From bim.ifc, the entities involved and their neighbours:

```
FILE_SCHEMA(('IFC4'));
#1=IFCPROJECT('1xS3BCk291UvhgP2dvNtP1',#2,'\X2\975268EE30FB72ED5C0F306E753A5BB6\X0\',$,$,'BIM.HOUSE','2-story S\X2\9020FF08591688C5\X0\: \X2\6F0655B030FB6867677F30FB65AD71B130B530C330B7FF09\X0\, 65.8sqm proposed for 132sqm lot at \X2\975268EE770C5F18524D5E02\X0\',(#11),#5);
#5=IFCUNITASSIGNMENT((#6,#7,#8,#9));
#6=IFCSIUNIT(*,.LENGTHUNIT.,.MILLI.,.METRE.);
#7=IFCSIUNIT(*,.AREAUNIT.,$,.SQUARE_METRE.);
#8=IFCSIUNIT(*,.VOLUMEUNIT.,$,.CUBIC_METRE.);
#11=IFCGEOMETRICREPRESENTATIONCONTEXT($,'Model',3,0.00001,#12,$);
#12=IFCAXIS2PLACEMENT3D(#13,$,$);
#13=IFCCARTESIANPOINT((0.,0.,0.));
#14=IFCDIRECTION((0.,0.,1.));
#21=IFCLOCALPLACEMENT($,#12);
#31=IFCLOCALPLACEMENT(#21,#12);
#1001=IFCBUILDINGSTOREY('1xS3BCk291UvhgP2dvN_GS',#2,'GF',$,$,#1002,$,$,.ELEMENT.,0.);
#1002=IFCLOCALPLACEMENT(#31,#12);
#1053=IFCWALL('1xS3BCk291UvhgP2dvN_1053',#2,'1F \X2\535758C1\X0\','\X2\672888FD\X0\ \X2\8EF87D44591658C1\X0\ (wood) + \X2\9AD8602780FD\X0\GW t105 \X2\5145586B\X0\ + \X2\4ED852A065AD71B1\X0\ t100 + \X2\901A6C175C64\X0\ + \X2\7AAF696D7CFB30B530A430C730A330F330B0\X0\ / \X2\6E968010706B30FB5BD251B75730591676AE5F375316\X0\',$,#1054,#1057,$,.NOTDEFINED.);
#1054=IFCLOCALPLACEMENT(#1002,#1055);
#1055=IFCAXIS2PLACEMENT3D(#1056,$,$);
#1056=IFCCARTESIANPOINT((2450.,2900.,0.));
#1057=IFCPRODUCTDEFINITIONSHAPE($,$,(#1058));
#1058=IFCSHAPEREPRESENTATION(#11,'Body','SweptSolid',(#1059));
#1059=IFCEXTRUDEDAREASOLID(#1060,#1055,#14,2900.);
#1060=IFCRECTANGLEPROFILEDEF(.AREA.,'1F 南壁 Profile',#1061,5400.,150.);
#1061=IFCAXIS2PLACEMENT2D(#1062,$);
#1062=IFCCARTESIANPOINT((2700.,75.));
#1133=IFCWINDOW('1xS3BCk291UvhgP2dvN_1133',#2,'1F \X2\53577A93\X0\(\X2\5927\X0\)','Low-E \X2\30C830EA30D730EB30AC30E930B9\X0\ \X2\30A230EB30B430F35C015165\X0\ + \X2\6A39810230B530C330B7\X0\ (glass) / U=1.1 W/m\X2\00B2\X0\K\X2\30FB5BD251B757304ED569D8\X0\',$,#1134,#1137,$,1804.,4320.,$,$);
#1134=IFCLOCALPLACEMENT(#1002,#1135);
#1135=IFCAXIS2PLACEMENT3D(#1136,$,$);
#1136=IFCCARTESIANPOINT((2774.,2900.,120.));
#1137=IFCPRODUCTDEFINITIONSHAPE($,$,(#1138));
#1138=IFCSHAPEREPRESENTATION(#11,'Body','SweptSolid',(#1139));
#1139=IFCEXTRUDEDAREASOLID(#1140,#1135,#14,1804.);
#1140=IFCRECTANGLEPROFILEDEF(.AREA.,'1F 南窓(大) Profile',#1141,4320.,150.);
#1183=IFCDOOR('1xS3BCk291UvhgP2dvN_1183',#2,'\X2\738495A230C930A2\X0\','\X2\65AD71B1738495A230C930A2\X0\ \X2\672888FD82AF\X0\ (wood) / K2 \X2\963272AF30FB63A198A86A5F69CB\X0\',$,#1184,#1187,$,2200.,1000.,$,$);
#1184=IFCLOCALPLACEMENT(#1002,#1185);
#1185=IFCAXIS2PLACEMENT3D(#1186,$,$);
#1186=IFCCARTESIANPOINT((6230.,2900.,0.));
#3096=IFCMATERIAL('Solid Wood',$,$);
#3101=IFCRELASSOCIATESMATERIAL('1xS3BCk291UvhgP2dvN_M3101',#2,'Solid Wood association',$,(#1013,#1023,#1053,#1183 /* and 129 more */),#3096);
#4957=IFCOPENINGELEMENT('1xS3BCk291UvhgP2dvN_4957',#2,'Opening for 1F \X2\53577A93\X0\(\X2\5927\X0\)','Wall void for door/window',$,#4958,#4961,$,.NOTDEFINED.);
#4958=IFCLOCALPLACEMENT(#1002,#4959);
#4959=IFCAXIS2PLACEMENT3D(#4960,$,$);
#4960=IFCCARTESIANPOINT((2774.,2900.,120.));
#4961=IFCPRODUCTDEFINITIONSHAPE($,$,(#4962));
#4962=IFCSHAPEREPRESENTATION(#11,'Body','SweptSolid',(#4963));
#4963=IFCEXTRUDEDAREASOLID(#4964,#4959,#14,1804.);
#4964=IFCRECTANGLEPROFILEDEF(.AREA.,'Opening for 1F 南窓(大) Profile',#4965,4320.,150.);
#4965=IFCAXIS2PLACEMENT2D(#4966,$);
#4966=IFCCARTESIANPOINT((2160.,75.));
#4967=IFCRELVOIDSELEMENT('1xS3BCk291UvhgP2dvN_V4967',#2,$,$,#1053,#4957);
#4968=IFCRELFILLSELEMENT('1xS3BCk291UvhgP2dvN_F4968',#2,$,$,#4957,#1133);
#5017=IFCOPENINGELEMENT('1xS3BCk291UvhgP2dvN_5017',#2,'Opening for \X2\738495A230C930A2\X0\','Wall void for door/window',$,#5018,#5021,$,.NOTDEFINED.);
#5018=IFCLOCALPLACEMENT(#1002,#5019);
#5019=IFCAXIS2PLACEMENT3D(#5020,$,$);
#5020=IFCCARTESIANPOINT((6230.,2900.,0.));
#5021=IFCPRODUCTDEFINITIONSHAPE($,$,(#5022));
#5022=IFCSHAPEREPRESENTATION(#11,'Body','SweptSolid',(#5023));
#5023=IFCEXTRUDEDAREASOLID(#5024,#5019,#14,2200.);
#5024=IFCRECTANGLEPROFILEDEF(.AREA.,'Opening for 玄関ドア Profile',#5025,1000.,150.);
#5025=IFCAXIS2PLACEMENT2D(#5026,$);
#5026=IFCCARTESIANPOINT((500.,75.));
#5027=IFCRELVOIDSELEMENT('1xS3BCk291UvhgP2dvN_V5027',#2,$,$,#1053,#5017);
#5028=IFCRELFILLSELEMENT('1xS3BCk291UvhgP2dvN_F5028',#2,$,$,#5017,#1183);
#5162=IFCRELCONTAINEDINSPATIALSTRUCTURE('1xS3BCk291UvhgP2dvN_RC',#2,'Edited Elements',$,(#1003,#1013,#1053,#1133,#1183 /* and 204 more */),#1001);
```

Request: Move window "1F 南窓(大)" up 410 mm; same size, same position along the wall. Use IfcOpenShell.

```python
import numpy as np
import ifcopenshell
import ifcopenshell.api.geometry
import ifcopenshell.util.placement
import ifcopenshell.util.unit

model = ifcopenshell.open("bim.ifc")
unit_scale = ifcopenshell.util.unit.calculate_unit_scale(model)

window = model.by_guid("1xS3BCk291UvhgP2dvN_1133")
opening = window.FillsVoids[0].RelatingOpeningElement
dz = 0.41 / unit_scale

shift = np.array([0.0, 0.0, dz])
# The window is not placed relative to its opening, so move both.
for product in (opening, window):
    matrix = ifcopenshell.util.placement.get_local_placement(product.ObjectPlacement)
    matrix[:3, 3] += shift
    ifcopenshell.api.geometry.edit_object_placement(model, product=product, matrix=matrix, is_si=False)

print(f"moved by {dz * unit_scale:+.3f} m")

model.write("bim_edited.ifc")
```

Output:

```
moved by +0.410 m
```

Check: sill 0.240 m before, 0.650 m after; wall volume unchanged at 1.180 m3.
